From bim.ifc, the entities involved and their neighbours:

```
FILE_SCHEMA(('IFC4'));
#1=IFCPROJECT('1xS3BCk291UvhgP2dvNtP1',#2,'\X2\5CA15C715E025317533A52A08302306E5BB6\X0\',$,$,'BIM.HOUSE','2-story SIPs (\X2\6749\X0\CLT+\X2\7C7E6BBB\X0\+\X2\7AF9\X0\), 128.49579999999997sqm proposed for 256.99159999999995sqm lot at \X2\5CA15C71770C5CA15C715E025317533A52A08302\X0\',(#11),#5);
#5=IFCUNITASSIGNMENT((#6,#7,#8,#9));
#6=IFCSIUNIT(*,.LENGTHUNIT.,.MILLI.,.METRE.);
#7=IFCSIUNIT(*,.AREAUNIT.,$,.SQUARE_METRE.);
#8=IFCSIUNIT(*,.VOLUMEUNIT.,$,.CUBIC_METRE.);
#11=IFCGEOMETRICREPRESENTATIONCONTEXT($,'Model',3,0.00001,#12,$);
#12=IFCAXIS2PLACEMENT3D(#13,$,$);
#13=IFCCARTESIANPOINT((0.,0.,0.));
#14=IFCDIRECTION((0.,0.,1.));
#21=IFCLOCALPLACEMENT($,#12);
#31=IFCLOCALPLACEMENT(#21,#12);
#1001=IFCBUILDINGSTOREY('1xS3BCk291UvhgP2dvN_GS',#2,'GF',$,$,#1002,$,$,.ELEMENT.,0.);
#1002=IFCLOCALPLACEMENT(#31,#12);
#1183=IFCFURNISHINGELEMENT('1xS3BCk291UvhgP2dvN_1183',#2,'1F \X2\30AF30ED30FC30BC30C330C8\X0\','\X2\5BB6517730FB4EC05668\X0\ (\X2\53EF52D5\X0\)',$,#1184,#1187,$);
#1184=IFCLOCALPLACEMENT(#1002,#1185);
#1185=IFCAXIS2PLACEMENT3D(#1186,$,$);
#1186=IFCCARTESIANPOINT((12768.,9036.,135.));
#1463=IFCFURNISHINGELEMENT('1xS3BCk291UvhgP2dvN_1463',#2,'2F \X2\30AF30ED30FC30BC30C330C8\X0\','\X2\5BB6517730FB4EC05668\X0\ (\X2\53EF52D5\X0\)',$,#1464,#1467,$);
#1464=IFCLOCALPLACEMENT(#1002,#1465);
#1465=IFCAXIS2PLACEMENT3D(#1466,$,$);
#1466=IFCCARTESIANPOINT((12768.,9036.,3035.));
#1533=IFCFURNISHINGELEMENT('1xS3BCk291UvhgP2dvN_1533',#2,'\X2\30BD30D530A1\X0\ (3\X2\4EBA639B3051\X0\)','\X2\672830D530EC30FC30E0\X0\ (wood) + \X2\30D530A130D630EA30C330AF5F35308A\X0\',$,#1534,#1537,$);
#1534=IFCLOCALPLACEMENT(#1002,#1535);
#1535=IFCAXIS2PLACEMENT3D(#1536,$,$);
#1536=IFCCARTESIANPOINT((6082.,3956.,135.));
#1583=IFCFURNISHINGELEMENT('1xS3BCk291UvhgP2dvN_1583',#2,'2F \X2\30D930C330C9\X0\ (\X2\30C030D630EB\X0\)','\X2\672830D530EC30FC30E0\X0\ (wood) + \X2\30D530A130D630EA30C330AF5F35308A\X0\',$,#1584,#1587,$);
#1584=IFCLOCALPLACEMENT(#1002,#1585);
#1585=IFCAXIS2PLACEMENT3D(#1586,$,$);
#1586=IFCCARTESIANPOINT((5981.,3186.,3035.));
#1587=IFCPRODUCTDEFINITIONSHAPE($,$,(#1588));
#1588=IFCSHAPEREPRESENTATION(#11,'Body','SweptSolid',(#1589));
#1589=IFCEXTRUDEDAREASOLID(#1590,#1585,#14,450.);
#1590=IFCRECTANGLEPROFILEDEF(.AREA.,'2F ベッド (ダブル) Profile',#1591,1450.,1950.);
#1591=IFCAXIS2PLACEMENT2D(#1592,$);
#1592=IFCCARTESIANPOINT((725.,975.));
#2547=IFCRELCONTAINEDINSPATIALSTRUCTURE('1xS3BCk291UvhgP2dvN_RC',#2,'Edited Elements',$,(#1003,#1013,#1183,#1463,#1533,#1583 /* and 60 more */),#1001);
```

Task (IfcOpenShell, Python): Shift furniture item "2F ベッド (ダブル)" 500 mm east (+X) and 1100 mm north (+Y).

```python
import ifcopenshell
import ifcopenshell.api.geometry
import ifcopenshell.util.placement
import ifcopenshell.util.unit

model = ifcopenshell.open("bim.ifc")
unit_scale = ifcopenshell.util.unit.calculate_unit_scale(model)

item = model.by_id(1583)
matrix = ifcopenshell.util.placement.get_local_placement(item.ObjectPlacement)
matrix[0, 3] += 0.5 / unit_scale
matrix[1, 3] += 1.1 / unit_scale
ifcopenshell.api.geometry.edit_object_placement(model, product=item, matrix=matrix, is_si=False)

print(ifcopenshell.util.placement.get_local_placement(item.ObjectPlacement).round(3) + 0.0)

model.write("bim_edited.ifc")
```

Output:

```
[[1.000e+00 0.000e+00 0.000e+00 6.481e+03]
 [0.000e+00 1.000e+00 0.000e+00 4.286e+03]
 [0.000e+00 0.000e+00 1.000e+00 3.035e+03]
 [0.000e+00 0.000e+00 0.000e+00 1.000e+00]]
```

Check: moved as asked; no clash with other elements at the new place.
